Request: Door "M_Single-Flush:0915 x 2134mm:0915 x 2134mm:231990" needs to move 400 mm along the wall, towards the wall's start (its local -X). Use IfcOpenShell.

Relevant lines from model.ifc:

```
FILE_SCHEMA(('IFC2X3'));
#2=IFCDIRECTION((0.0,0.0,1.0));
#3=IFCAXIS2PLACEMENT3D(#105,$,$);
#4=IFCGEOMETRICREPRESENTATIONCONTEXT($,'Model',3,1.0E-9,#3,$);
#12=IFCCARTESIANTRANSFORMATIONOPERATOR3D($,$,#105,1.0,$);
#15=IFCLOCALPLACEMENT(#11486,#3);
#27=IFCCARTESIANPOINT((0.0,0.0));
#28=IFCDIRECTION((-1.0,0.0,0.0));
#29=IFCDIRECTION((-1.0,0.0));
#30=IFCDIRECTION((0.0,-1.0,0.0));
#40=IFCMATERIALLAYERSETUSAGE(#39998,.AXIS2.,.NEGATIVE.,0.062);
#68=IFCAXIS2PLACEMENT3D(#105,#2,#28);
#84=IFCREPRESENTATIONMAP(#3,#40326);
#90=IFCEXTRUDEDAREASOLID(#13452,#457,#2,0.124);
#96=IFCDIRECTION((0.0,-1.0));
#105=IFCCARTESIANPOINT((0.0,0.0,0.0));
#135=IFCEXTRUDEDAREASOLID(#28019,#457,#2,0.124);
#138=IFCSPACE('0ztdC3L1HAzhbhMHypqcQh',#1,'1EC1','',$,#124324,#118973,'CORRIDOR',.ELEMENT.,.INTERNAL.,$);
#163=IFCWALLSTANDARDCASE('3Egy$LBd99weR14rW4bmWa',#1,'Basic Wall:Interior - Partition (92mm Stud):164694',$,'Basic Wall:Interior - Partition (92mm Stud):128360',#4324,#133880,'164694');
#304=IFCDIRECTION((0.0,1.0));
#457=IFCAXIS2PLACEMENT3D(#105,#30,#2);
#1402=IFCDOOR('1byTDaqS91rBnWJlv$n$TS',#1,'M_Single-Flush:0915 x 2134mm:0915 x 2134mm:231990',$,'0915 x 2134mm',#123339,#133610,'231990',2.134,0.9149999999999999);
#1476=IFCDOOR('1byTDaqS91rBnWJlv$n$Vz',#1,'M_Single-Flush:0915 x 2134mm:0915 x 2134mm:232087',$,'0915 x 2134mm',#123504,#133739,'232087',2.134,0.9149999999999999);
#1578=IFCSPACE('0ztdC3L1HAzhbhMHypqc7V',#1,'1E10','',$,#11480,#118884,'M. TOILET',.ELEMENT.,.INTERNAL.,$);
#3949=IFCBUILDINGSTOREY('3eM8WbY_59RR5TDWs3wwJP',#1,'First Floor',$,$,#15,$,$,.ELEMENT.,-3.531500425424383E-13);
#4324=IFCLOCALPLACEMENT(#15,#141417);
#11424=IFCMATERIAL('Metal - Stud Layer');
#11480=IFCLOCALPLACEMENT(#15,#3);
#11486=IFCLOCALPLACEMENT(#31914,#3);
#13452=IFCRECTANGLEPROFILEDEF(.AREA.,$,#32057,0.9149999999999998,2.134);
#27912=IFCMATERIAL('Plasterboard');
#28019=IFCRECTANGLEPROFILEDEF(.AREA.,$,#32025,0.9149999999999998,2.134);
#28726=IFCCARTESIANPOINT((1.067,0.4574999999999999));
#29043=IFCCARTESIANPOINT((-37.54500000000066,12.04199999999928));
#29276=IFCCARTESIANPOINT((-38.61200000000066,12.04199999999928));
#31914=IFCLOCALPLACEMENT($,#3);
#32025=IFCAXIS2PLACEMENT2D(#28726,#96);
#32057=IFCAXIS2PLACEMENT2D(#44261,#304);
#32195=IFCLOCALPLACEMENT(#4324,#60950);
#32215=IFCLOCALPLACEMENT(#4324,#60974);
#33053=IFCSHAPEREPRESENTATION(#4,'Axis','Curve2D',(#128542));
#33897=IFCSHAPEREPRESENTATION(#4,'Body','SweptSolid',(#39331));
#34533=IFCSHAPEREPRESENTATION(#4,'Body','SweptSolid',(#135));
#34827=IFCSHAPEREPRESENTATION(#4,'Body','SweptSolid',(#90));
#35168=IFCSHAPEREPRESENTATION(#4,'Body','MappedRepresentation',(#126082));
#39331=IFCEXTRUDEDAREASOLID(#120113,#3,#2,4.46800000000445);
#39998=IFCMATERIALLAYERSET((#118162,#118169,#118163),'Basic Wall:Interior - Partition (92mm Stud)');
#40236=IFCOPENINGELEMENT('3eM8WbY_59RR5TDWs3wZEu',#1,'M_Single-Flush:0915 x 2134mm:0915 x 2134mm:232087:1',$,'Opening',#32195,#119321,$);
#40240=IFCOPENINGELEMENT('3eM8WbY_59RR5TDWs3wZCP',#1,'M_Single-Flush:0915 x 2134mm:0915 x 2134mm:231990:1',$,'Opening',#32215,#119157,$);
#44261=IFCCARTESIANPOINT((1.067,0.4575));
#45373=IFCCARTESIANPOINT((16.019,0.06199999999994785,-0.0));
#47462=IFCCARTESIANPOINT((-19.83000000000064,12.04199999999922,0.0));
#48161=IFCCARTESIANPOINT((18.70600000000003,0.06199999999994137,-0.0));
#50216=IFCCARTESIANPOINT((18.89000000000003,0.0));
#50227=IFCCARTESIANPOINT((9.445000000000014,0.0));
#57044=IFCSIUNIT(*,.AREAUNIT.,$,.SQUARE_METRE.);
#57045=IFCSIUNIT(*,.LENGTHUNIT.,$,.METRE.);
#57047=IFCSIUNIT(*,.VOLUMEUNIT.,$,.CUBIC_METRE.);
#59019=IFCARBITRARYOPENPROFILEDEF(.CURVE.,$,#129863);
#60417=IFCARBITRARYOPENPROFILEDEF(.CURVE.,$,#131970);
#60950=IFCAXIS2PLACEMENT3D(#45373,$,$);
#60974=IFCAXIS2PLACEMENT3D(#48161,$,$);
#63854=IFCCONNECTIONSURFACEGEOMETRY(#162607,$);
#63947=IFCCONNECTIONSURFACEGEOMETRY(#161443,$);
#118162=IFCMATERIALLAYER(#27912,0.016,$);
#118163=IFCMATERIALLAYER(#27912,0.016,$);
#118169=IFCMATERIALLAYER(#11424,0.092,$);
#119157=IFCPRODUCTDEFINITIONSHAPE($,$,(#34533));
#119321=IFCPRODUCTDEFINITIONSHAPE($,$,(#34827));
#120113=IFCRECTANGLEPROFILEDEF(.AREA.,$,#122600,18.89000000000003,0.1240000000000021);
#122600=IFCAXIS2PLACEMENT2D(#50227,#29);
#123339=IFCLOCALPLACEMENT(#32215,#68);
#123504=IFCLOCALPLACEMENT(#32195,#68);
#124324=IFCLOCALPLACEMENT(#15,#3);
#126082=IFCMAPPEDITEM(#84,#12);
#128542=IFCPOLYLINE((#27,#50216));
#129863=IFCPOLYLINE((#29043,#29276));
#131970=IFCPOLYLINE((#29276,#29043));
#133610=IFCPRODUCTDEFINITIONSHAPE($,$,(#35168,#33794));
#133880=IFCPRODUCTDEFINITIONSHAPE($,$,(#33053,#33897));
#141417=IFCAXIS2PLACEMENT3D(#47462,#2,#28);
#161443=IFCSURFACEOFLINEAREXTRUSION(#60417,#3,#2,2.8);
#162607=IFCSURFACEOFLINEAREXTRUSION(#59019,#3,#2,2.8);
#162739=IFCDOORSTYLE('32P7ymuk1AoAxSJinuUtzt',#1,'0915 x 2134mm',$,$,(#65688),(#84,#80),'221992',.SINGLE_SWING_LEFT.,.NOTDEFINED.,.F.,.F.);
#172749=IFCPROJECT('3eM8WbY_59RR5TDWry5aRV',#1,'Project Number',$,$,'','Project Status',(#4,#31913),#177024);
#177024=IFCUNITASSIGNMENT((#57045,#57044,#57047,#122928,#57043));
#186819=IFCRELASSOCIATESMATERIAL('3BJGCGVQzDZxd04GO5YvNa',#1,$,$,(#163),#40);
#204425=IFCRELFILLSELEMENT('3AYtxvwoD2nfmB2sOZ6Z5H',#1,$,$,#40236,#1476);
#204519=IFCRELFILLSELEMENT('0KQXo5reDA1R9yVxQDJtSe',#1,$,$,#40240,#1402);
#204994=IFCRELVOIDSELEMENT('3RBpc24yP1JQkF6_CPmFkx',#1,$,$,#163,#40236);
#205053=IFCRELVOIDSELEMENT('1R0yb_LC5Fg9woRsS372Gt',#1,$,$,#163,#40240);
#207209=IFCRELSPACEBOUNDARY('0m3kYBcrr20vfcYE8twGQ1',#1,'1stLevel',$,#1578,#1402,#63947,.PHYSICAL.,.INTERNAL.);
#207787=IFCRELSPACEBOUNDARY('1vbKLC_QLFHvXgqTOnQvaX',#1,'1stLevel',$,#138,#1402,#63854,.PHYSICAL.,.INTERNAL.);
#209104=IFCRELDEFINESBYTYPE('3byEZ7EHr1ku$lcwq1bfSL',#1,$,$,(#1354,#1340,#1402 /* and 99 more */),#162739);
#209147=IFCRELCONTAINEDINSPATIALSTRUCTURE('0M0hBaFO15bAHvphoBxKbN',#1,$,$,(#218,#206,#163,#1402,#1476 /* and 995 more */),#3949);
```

```python
import numpy as np
import ifcopenshell
import ifcopenshell.api.geometry
import ifcopenshell.util.placement

model = ifcopenshell.open("model.ifc")

door = model.by_id(1402)
opening = door.FillsVoids[0].RelatingOpeningElement
wall = opening.VoidsElements[0].RelatingBuildingElement

wall_matrix = ifcopenshell.util.placement.get_local_placement(wall.ObjectPlacement)
shift = wall_matrix[:3, 0] * -0.4
before = ifcopenshell.util.placement.get_local_placement(door.ObjectPlacement)[:3, 3].copy()

# The door is placed relative to its opening, so it follows when the opening moves.
matrix = ifcopenshell.util.placement.get_local_placement(opening.ObjectPlacement)
matrix[:3, 3] += shift
ifcopenshell.api.geometry.edit_object_placement(
    model, product=opening, matrix=matrix, is_si=False, should_transform_children=True
)

# Space boundary surfaces are stored in each space's coordinates; move them too.
for rel in door.ProvidesBoundaries:
    if not rel.ConnectionGeometry:
        continue
    surface = rel.ConnectionGeometry.SurfaceOnRelatingElement
    space_matrix = ifcopenshell.util.placement.get_local_placement(rel.RelatingSpace.ObjectPlacement)
    point = np.array(surface.Position.Location.Coordinates) + space_matrix[:3, :3].T @ shift
    surface.Position = model.createIfcAxis2Placement3D(
        model.createIfcCartesianPoint(point.tolist()), surface.Position.Axis, surface.Position.RefDirection
    )

after = ifcopenshell.util.placement.get_local_placement(door.ObjectPlacement)[:3, 3]
print("door moved by", (after - before).round(3) + 0.0)

model.write("model-out.ifc")
```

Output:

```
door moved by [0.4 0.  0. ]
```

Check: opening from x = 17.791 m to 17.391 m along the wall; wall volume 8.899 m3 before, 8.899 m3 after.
